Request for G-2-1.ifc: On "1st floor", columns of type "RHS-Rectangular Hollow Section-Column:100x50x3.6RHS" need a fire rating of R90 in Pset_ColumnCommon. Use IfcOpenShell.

First a look at what the model holds.

```python
import ifcopenshell
import ifcopenshell.util.element

model = ifcopenshell.open("G-2-1.ifc")
print(model.schema)
storey = next(s for s in model.by_type("IfcBuildingStorey") if s.Name == "1st floor")
columns = [e for e in ifcopenshell.util.element.get_decomposition(storey) if e.is_a("IfcColumn")]
seen = {}
for e in columns:
    element_type = ifcopenshell.util.element.get_type(e)
    key = (element_type.Name if element_type != e and element_type else None, ifcopenshell.util.element.get_pset(e, "Pset_ColumnCommon", "FireRating"))
    seen[key] = seen.get(key, 0) + 1
for (name, value), count in sorted(seen.items(), key=str):
    print(count, "x", name, "|", value)
```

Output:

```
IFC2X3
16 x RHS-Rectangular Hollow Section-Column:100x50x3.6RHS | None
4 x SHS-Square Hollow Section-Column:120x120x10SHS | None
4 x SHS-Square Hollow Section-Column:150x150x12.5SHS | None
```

```python
import ifcopenshell
import ifcopenshell.api.pset
import ifcopenshell.util.element

model = ifcopenshell.open("G-2-1.ifc")

storey = next(s for s in model.by_type("IfcBuildingStorey") if s.Name == "1st floor")
columns = [e for e in ifcopenshell.util.element.get_decomposition(storey) if e.is_a("IfcColumn")]

count = 0
for e in columns:
    element_type = ifcopenshell.util.element.get_type(e)
    if element_type in (None, e) or element_type.Name != "RHS-Rectangular Hollow Section-Column:100x50x3.6RHS":
        continue
    # add_pset returns the element's existing set when there is one.
    pset = ifcopenshell.api.pset.add_pset(model, product=e, name="Pset_ColumnCommon")
    ifcopenshell.api.pset.edit_pset(model, pset=pset, properties={"FireRating": "R90"})
    count += 1

print(count, "columns updated")

model.write("G-2-1_v2.ifc")
```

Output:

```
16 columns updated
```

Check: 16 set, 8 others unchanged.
